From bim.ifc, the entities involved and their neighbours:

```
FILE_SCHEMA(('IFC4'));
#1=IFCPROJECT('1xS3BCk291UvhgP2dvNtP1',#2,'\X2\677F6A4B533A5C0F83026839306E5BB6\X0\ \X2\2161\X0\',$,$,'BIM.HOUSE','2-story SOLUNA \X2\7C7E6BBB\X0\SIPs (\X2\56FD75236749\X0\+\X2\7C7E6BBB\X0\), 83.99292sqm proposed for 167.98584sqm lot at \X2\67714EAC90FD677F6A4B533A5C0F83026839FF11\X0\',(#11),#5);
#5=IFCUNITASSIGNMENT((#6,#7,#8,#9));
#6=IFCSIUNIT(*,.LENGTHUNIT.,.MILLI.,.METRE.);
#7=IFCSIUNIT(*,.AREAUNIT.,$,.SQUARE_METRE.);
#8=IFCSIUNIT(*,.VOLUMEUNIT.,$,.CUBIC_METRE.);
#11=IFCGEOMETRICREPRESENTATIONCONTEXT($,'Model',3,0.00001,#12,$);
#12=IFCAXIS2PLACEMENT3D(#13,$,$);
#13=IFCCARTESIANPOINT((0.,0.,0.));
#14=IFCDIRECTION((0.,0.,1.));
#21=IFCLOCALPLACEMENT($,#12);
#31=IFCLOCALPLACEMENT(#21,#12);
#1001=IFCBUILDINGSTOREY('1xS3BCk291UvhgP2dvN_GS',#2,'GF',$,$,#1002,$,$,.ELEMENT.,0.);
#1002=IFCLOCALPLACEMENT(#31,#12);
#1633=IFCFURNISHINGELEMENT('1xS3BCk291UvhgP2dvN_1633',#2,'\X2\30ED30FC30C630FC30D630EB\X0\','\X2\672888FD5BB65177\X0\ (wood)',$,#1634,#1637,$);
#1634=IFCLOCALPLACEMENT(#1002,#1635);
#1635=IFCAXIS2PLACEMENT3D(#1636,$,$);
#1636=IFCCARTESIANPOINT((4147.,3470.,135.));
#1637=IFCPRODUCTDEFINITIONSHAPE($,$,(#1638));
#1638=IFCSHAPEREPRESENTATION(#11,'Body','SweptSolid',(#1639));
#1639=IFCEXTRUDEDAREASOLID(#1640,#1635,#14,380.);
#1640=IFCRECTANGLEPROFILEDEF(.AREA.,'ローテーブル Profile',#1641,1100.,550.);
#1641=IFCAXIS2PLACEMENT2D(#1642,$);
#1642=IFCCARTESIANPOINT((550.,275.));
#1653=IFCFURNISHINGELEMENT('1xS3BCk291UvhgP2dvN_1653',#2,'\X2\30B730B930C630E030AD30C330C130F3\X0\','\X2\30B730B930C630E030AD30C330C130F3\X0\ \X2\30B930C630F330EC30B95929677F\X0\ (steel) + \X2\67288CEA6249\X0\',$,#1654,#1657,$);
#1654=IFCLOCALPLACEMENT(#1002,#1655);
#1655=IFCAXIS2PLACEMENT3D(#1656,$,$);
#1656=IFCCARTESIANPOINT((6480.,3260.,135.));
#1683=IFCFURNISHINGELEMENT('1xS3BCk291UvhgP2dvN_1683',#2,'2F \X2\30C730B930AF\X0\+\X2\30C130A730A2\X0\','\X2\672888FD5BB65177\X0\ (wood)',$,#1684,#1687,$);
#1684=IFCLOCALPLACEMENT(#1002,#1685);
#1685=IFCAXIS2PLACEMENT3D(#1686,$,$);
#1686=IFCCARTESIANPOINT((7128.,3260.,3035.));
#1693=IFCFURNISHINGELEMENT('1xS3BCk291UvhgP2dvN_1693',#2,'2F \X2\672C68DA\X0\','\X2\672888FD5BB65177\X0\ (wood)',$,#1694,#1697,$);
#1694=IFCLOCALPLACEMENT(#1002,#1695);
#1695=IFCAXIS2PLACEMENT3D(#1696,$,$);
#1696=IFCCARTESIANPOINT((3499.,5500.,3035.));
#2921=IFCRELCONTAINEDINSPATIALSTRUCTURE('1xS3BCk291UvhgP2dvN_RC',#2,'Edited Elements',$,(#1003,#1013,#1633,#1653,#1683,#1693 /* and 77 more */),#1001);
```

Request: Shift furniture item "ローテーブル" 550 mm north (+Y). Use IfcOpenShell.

```python
import ifcopenshell
import ifcopenshell.api.geometry
import ifcopenshell.util.placement
import ifcopenshell.util.unit

model = ifcopenshell.open("bim.ifc")
unit_scale = ifcopenshell.util.unit.calculate_unit_scale(model)

item = model.by_guid("1xS3BCk291UvhgP2dvN_1633")
matrix = ifcopenshell.util.placement.get_local_placement(item.ObjectPlacement)
matrix[1, 3] += 0.55 / unit_scale
ifcopenshell.api.geometry.edit_object_placement(model, product=item, matrix=matrix, is_si=False)

print(ifcopenshell.util.placement.get_local_placement(item.ObjectPlacement).round(3) + 0.0)

model.write("bim_updated.ifc")
```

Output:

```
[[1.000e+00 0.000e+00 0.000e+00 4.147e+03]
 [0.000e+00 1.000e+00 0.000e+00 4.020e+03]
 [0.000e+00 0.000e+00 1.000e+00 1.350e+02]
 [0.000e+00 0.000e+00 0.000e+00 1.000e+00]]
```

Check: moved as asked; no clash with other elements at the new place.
